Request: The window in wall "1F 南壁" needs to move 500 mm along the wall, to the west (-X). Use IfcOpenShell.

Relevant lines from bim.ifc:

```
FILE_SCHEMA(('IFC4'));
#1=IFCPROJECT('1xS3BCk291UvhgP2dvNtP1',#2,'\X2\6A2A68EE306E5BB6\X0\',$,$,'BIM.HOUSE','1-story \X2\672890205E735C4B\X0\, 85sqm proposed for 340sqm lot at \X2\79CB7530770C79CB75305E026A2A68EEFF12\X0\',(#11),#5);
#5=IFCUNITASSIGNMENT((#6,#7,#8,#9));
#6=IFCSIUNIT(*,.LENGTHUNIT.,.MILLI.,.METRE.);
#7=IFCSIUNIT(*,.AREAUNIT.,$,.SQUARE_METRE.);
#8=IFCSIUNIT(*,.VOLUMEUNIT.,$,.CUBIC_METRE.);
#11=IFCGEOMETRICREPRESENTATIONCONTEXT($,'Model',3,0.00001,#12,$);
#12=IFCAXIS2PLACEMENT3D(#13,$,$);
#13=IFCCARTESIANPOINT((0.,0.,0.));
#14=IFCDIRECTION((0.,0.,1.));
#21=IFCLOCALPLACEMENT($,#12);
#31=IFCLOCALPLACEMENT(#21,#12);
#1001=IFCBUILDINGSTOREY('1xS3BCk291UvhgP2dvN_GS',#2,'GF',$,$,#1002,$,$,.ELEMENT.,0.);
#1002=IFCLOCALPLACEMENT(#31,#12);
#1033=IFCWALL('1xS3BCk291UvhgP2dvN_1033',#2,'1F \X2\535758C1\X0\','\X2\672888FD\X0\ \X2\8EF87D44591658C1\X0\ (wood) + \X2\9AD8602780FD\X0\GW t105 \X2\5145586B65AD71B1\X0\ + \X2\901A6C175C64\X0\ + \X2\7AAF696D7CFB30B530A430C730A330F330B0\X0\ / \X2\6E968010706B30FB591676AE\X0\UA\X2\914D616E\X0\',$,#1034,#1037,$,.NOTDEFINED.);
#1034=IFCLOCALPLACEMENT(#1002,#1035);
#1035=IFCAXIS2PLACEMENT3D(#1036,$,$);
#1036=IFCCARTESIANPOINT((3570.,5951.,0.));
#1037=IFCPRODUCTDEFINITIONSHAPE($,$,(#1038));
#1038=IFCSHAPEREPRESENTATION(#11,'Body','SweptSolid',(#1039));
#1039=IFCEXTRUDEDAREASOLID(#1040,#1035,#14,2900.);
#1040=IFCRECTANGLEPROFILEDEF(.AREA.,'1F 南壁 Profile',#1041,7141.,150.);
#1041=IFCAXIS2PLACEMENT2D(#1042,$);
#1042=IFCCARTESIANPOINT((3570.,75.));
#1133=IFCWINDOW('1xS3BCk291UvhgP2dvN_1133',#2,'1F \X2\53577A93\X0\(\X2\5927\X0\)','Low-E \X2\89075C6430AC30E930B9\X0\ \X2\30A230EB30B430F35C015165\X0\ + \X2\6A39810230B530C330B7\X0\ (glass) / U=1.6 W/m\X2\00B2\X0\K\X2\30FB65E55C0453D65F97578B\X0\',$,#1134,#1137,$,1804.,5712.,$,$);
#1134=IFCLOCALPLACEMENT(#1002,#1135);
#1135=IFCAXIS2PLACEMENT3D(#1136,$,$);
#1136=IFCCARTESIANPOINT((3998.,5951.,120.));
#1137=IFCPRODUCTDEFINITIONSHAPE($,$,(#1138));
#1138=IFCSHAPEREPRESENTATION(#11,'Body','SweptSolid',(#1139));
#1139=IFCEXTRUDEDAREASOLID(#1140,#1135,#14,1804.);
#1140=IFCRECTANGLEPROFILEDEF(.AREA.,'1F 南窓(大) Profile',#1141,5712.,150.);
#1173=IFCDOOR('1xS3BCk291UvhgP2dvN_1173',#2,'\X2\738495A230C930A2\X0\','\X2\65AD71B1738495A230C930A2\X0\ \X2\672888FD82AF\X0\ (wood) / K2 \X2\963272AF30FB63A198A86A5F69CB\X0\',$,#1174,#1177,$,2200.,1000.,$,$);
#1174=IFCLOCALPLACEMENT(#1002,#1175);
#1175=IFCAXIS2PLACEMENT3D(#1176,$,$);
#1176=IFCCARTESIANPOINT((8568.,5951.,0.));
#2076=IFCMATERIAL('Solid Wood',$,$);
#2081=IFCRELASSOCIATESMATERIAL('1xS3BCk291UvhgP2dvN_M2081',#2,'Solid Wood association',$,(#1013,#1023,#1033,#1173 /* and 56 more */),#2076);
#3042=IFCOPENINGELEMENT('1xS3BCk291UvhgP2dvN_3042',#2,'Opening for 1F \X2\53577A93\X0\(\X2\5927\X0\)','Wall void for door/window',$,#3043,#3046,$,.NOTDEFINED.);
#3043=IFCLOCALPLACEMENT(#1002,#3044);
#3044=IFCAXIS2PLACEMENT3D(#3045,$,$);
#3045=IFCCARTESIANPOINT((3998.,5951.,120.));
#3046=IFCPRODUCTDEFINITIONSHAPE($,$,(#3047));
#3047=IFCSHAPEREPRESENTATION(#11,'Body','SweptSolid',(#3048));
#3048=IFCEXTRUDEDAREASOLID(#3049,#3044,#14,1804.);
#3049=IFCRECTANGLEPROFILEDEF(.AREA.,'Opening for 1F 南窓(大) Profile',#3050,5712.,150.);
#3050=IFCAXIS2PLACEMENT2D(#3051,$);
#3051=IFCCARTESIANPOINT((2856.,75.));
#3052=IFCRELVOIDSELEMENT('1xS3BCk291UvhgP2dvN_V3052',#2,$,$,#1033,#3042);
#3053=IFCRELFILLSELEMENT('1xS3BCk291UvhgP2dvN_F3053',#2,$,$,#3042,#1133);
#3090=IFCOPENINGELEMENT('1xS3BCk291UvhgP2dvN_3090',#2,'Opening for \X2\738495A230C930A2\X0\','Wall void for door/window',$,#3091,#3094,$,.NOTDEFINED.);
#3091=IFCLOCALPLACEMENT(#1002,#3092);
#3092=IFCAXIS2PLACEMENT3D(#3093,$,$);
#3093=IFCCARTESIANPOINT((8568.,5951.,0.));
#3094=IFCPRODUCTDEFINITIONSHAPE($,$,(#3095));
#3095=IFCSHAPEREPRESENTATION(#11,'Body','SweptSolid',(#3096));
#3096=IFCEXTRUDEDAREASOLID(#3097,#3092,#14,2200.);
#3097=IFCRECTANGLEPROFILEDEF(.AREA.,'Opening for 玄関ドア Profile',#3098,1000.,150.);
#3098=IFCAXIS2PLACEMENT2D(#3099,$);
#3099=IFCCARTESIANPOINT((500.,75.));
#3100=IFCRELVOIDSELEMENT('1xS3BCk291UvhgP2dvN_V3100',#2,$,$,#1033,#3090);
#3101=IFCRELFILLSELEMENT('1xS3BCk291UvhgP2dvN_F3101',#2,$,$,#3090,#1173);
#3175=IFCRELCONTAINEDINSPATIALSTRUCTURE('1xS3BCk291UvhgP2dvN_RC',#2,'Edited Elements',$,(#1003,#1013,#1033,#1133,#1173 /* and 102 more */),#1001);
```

```python
import ifcopenshell
import ifcopenshell.api.geometry
import ifcopenshell.util.placement
import ifcopenshell.util.unit

model = ifcopenshell.open("bim.ifc")
unit_scale = ifcopenshell.util.unit.calculate_unit_scale(model)

window = model.by_guid("1xS3BCk291UvhgP2dvN_1133")
opening = window.FillsVoids[0].RelatingOpeningElement
wall = opening.VoidsElements[0].RelatingBuildingElement

wall_matrix = ifcopenshell.util.placement.get_local_placement(wall.ObjectPlacement)
shift = wall_matrix[:3, 0] * -0.5 / unit_scale
before = ifcopenshell.util.placement.get_local_placement(window.ObjectPlacement)[:3, 3].copy()

# The window is not placed relative to its opening, so move both.
for product in (opening, window):
    matrix = ifcopenshell.util.placement.get_local_placement(product.ObjectPlacement)
    matrix[:3, 3] += shift
    ifcopenshell.api.geometry.edit_object_placement(model, product=product, matrix=matrix, is_si=False)

after = ifcopenshell.util.placement.get_local_placement(window.ObjectPlacement)[:3, 3]
print("window moved by", (after - before).round(3) + 0.0)

model.write("bim_v2.ifc")
```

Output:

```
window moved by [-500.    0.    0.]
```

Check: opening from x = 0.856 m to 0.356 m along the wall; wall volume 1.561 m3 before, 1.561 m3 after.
